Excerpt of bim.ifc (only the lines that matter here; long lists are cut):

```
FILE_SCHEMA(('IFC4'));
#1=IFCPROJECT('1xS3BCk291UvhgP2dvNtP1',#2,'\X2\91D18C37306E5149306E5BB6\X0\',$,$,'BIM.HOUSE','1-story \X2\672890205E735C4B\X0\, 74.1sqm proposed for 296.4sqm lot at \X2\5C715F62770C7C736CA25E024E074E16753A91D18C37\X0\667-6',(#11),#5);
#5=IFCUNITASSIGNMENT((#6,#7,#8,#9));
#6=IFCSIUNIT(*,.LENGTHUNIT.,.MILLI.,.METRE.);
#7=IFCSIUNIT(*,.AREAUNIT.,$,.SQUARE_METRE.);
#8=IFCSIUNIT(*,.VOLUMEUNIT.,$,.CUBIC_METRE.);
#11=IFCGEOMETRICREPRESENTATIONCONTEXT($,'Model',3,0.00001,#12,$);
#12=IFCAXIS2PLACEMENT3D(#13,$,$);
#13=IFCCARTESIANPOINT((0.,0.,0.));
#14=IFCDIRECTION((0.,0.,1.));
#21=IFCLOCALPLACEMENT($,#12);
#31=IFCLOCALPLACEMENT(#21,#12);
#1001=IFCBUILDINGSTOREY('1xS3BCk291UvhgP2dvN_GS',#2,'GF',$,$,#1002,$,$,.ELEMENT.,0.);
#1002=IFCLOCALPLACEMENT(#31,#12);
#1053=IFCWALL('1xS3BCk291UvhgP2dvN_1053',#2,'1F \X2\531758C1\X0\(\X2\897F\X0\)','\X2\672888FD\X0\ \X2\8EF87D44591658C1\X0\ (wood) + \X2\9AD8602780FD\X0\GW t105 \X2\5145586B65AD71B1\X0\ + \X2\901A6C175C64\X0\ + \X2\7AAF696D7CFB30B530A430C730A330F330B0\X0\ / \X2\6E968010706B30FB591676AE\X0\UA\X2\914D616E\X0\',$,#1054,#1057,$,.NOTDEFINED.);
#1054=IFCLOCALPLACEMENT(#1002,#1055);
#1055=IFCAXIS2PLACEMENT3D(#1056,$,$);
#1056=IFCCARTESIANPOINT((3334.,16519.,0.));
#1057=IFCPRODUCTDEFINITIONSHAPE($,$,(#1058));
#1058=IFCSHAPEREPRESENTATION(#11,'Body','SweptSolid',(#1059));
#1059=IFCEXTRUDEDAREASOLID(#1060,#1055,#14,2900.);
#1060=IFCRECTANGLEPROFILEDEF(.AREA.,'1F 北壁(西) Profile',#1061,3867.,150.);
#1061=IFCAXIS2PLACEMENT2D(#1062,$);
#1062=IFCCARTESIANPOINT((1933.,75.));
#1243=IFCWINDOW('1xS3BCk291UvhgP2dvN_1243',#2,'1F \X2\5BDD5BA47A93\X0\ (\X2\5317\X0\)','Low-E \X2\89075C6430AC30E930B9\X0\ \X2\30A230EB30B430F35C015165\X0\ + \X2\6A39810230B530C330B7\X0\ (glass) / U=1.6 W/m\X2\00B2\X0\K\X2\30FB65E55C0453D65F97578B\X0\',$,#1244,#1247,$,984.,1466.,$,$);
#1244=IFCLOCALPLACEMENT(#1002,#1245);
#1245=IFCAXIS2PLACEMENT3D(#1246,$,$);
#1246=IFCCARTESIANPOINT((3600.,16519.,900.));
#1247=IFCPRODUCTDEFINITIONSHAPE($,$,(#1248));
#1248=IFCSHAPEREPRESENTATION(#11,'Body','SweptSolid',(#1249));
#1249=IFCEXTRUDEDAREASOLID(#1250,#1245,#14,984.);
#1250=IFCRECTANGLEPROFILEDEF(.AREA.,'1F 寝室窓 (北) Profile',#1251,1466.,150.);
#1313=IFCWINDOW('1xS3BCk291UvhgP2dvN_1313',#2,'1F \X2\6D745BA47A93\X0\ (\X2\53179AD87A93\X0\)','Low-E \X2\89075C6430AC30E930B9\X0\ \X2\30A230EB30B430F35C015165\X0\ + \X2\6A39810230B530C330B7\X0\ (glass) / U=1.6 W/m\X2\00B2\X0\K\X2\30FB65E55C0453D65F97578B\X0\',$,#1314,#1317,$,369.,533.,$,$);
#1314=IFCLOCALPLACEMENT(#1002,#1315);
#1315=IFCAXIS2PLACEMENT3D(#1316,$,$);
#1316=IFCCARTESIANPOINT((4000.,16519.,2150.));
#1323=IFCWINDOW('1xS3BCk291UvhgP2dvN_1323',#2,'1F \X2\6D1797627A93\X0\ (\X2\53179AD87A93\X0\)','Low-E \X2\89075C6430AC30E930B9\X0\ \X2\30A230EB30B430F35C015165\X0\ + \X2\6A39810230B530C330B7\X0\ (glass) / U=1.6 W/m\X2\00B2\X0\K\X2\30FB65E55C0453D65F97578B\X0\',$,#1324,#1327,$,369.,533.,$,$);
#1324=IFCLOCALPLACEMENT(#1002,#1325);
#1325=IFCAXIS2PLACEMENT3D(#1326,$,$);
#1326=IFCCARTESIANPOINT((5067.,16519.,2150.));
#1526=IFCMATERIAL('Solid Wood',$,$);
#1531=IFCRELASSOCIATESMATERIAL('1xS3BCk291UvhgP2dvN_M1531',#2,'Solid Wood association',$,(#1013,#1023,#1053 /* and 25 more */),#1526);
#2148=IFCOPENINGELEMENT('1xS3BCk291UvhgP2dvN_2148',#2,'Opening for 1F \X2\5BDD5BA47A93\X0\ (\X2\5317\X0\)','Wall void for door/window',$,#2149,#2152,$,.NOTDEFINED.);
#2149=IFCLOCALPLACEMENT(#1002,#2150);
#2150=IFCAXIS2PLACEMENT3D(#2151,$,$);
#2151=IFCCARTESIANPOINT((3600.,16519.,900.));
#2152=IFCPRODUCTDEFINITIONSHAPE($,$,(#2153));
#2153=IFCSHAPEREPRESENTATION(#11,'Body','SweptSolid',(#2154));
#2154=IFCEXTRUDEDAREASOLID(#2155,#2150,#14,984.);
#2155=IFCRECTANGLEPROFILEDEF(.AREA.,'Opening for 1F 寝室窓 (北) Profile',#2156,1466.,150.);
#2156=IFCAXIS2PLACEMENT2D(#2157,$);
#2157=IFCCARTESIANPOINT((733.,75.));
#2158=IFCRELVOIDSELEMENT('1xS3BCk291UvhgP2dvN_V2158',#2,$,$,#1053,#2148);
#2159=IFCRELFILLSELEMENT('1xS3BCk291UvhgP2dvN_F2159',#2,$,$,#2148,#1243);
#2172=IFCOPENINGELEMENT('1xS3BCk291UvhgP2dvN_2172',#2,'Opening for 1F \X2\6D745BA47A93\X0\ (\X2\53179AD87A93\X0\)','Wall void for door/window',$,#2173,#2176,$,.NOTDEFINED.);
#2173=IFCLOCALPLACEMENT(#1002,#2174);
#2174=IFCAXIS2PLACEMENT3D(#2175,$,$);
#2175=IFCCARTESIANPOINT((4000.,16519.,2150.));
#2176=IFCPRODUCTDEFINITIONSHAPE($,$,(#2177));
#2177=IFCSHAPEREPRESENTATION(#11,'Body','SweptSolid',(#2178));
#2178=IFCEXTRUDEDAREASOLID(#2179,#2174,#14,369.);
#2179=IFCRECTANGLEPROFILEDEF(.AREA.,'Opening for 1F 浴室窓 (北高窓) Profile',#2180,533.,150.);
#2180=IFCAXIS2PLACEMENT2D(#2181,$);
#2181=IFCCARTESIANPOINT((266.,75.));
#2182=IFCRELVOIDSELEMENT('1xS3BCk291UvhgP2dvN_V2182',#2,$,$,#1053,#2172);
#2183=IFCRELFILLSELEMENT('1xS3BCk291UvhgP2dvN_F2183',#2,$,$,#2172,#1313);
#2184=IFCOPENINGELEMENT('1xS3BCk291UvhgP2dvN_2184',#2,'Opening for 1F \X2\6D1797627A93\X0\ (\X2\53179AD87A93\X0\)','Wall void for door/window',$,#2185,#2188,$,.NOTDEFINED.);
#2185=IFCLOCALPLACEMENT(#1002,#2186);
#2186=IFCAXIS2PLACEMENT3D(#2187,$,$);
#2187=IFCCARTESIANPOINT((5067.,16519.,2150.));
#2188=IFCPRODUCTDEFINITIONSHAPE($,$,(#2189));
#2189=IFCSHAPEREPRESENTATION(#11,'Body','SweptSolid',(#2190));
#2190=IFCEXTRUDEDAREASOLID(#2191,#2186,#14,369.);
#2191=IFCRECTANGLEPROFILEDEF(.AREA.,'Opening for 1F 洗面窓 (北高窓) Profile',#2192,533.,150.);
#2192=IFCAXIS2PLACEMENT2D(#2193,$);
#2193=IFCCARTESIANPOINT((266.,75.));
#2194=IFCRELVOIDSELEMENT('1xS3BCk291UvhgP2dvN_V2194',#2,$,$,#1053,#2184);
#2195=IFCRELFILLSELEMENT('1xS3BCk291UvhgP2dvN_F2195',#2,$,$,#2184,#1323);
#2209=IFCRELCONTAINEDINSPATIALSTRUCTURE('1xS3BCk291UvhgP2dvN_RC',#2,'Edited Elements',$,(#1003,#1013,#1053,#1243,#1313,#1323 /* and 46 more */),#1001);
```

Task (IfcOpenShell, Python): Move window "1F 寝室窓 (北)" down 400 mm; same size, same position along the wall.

```python
import numpy as np
import ifcopenshell
import ifcopenshell.api.geometry
import ifcopenshell.util.placement
import ifcopenshell.util.unit

model = ifcopenshell.open("bim.ifc")
unit_scale = ifcopenshell.util.unit.calculate_unit_scale(model)

window = model.by_id(1243)
opening = window.FillsVoids[0].RelatingOpeningElement
dz = -400.0

shift = np.array([0.0, 0.0, dz])
# The window is not placed relative to its opening, so move both.
for product in (opening, window):
    matrix = ifcopenshell.util.placement.get_local_placement(product.ObjectPlacement)
    matrix[:3, 3] += shift
    ifcopenshell.api.geometry.edit_object_placement(model, product=product, matrix=matrix, is_si=False)

print(f"moved by {dz * unit_scale:+.3f} m")

model.write("bim-out.ifc")
```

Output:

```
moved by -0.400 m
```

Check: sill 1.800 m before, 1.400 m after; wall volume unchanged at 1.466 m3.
